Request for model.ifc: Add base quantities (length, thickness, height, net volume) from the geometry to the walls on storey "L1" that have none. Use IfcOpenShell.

First a look at what the model holds.

```python
import ifcopenshell
import ifcopenshell.util.element
import ifcopenshell.util.unit

model = ifcopenshell.open("model.ifc")
print(model.schema)
for unit_type in ("LENGTHUNIT", "AREAUNIT", "VOLUMEUNIT"):
    print(unit_type, ifcopenshell.util.unit.calculate_unit_scale(model, unit_type))
storey = next(s for s in model.by_type("IfcBuildingStorey") if s.Name == "L1")
walls = [e for e in ifcopenshell.util.element.get_decomposition(storey) if e.is_a("IfcWall")]
for e in sorted(walls, key=lambda e: e.id()):
    print(e.id(), e.is_a(), e.Name, list(ifcopenshell.util.element.get_psets(e, qtos_only=True)), sep=" | ")
```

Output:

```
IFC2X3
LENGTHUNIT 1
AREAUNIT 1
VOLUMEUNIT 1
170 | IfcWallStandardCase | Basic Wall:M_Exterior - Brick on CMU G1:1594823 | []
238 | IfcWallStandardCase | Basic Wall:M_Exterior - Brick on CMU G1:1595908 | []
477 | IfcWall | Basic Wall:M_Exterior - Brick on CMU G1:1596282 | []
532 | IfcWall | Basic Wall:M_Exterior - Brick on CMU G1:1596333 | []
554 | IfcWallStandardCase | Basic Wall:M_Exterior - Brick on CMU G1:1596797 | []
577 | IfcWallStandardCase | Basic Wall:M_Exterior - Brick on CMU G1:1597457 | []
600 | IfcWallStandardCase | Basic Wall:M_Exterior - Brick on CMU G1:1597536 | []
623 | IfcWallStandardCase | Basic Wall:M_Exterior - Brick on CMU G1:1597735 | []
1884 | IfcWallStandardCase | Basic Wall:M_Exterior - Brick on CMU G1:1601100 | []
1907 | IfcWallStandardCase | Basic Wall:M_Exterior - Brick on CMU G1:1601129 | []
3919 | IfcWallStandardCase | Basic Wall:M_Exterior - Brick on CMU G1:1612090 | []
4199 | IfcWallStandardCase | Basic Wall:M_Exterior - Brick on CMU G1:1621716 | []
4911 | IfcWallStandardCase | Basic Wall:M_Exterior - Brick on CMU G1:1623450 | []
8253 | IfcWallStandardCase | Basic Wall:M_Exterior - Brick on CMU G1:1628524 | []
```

```python
import ifcopenshell
import ifcopenshell.api.pset
import ifcopenshell.geom
import ifcopenshell.util.element
import ifcopenshell.util.shape
import ifcopenshell.util.unit

model = ifcopenshell.open("model.ifc")
unit_scale = ifcopenshell.util.unit.calculate_unit_scale(model)
volume_scale = ifcopenshell.util.unit.calculate_unit_scale(model, "VOLUMEUNIT")
settings = ifcopenshell.geom.settings()

storey = next(s for s in model.by_type("IfcBuildingStorey") if s.Name == "L1")
walls = [e for e in ifcopenshell.util.element.get_decomposition(storey) if e.is_a("IfcWall")]

for e in sorted(walls, key=lambda e: e.id()):
    if ifcopenshell.util.element.get_psets(e, qtos_only=True, should_inherit=False):
        continue
    # Geometry comes back in metres, in the element's own axes.
    shape = ifcopenshell.geom.create_shape(settings, e)
    values = {
        "Length": ifcopenshell.util.shape.get_x(shape.geometry) / unit_scale,
        "Width": ifcopenshell.util.shape.get_y(shape.geometry) / unit_scale,
        "Height": ifcopenshell.util.shape.get_z(shape.geometry) / unit_scale,
        "NetVolume": ifcopenshell.util.shape.get_volume(shape.geometry) / volume_scale,
    }
    qto = ifcopenshell.api.pset.add_qto(model, product=e, name="BaseQuantities")
    ifcopenshell.api.pset.edit_qto(model, qto=qto, properties=values)
    print(e.id(), {k: round(v, 3) for k, v in values.items()})

model.write("model-out.ifc")
```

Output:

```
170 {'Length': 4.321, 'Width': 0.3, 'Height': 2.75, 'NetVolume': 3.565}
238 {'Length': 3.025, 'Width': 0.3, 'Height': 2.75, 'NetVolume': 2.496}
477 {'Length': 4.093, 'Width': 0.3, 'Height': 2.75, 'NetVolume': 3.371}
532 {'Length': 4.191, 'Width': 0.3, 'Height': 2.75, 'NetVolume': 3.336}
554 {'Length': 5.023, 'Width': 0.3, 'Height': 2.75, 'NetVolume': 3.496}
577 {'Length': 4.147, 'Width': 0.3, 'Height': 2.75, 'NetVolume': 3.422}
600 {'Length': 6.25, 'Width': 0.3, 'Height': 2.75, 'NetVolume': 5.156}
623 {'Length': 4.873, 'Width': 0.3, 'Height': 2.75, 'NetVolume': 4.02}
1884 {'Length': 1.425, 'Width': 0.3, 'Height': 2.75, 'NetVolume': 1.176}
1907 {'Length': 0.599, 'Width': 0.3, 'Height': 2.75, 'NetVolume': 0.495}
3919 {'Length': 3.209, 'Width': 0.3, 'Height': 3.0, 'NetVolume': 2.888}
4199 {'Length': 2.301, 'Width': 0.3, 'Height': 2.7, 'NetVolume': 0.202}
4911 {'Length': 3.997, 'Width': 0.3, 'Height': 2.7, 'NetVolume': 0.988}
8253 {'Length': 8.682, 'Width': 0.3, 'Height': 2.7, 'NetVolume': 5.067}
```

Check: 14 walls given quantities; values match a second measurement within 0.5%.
